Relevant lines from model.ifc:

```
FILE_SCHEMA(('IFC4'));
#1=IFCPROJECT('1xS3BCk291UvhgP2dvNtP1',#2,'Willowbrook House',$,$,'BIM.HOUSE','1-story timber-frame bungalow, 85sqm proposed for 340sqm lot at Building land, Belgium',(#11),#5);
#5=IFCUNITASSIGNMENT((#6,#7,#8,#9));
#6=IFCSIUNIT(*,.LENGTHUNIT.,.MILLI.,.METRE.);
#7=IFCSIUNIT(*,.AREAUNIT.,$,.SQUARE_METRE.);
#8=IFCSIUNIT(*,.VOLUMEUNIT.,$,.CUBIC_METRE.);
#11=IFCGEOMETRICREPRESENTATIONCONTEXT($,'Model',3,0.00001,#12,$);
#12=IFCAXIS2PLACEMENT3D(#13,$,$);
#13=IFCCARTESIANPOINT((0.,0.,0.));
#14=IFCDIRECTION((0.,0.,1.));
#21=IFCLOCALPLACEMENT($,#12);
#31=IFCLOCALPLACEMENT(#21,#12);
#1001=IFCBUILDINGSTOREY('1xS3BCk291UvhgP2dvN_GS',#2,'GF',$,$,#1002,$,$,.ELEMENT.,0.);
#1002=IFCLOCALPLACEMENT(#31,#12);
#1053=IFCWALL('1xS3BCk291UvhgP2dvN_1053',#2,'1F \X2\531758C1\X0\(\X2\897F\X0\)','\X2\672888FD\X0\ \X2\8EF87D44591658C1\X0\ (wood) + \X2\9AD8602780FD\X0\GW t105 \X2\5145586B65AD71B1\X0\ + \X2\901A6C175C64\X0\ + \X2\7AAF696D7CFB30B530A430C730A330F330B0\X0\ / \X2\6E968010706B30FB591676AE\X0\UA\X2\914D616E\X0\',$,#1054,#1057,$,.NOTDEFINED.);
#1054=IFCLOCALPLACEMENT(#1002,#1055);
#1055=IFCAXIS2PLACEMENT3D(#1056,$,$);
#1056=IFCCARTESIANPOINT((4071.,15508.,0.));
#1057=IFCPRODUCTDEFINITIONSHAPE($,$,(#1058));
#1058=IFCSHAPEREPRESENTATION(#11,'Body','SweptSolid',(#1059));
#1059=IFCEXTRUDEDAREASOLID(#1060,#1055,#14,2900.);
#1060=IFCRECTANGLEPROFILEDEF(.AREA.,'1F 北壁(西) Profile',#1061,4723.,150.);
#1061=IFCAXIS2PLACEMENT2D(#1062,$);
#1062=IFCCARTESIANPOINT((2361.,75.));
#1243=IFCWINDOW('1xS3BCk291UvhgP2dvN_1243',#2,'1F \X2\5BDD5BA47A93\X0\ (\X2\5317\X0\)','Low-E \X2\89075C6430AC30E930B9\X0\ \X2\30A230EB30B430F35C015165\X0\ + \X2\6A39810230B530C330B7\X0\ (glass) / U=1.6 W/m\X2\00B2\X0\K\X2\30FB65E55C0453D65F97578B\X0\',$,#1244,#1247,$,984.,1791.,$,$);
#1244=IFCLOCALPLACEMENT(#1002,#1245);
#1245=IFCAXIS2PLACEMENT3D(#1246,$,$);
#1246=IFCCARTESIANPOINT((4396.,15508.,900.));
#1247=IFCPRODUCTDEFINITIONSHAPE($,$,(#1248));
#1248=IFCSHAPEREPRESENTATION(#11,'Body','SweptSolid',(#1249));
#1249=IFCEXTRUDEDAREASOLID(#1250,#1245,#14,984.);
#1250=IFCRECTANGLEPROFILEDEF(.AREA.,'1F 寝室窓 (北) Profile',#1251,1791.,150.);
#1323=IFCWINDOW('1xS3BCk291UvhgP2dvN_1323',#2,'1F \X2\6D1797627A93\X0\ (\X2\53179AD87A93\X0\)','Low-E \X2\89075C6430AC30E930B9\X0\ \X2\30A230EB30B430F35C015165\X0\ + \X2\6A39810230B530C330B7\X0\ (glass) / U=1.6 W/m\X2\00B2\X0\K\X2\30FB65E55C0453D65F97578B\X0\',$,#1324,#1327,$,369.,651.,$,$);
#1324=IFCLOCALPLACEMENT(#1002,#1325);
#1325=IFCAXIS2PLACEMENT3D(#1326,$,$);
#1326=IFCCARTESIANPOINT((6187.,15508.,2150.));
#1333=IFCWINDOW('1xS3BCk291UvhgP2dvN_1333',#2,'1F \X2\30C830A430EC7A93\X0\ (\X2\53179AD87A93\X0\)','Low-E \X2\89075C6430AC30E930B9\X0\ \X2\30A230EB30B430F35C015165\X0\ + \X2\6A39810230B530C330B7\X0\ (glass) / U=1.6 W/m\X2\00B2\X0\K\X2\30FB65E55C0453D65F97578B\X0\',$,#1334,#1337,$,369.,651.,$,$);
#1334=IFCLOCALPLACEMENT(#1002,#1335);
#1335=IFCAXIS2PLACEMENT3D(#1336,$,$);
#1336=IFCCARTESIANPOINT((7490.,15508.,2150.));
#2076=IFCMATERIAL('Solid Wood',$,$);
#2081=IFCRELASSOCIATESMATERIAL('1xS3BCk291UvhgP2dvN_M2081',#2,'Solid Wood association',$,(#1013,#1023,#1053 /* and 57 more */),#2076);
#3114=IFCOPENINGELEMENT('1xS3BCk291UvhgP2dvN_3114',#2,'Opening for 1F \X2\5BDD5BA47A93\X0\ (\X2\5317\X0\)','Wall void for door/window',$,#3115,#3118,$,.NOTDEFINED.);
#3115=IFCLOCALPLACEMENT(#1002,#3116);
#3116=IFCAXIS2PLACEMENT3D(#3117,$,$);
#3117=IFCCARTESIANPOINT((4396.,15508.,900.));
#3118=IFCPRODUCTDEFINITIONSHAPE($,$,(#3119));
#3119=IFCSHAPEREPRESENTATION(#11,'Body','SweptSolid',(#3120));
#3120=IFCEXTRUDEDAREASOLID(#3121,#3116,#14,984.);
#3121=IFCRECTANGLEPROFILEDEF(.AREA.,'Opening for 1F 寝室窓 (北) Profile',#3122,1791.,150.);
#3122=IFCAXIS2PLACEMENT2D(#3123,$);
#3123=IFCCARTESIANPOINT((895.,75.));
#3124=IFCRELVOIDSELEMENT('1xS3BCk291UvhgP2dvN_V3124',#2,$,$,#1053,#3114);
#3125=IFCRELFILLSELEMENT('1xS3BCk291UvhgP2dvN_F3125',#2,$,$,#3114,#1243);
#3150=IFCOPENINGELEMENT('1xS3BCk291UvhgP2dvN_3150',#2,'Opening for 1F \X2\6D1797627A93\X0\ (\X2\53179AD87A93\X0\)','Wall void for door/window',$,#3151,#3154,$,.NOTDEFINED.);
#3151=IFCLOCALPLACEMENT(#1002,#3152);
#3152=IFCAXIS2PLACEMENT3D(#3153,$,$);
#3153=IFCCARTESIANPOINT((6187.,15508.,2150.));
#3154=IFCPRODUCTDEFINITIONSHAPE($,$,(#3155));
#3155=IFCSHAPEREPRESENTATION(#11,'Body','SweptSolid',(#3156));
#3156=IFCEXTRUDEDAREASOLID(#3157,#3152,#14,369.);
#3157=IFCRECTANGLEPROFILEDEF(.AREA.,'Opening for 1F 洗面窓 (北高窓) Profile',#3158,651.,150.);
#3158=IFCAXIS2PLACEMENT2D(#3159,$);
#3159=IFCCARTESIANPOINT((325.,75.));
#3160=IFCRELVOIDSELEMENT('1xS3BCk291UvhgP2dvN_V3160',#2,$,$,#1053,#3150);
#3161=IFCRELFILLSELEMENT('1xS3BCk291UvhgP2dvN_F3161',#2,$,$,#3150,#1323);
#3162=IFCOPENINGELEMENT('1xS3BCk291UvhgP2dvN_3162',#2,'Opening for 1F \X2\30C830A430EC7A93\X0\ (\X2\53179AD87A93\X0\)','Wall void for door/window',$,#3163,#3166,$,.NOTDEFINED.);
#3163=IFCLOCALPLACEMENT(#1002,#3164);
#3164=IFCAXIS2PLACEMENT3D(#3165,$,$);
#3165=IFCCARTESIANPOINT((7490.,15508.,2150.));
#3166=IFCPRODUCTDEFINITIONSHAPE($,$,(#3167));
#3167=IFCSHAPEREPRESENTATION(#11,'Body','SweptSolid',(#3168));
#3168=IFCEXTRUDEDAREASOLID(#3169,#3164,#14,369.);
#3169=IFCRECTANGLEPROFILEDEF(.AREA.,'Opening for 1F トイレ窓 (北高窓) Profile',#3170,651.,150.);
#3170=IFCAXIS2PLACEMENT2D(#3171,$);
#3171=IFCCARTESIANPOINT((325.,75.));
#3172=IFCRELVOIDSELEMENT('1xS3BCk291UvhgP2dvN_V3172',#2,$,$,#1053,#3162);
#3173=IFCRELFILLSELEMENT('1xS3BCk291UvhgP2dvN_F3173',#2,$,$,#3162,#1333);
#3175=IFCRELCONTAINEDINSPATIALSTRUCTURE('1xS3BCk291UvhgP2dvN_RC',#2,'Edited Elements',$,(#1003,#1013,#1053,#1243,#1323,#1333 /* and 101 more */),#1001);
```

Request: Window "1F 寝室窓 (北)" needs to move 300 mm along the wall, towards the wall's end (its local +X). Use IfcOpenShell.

```python
import ifcopenshell
import ifcopenshell.api.geometry
import ifcopenshell.util.placement
import ifcopenshell.util.unit

model = ifcopenshell.open("model.ifc")
unit_scale = ifcopenshell.util.unit.calculate_unit_scale(model)

window = model.by_guid("1xS3BCk291UvhgP2dvN_1243")
opening = window.FillsVoids[0].RelatingOpeningElement
wall = opening.VoidsElements[0].RelatingBuildingElement

wall_matrix = ifcopenshell.util.placement.get_local_placement(wall.ObjectPlacement)
shift = wall_matrix[:3, 0] * 0.3 / unit_scale
before = ifcopenshell.util.placement.get_local_placement(window.ObjectPlacement)[:3, 3].copy()

# The window is not placed relative to its opening, so move both.
for product in (opening, window):
    matrix = ifcopenshell.util.placement.get_local_placement(product.ObjectPlacement)
    matrix[:3, 3] += shift
    ifcopenshell.api.geometry.edit_object_placement(model, product=product, matrix=matrix, is_si=False)

after = ifcopenshell.util.placement.get_local_placement(window.ObjectPlacement)[:3, 3]
print("window moved by", (after - before).round(3) + 0.0)

model.write("model_edited.ifc")
```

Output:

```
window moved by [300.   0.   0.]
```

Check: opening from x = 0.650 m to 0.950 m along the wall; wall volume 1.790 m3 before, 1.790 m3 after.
